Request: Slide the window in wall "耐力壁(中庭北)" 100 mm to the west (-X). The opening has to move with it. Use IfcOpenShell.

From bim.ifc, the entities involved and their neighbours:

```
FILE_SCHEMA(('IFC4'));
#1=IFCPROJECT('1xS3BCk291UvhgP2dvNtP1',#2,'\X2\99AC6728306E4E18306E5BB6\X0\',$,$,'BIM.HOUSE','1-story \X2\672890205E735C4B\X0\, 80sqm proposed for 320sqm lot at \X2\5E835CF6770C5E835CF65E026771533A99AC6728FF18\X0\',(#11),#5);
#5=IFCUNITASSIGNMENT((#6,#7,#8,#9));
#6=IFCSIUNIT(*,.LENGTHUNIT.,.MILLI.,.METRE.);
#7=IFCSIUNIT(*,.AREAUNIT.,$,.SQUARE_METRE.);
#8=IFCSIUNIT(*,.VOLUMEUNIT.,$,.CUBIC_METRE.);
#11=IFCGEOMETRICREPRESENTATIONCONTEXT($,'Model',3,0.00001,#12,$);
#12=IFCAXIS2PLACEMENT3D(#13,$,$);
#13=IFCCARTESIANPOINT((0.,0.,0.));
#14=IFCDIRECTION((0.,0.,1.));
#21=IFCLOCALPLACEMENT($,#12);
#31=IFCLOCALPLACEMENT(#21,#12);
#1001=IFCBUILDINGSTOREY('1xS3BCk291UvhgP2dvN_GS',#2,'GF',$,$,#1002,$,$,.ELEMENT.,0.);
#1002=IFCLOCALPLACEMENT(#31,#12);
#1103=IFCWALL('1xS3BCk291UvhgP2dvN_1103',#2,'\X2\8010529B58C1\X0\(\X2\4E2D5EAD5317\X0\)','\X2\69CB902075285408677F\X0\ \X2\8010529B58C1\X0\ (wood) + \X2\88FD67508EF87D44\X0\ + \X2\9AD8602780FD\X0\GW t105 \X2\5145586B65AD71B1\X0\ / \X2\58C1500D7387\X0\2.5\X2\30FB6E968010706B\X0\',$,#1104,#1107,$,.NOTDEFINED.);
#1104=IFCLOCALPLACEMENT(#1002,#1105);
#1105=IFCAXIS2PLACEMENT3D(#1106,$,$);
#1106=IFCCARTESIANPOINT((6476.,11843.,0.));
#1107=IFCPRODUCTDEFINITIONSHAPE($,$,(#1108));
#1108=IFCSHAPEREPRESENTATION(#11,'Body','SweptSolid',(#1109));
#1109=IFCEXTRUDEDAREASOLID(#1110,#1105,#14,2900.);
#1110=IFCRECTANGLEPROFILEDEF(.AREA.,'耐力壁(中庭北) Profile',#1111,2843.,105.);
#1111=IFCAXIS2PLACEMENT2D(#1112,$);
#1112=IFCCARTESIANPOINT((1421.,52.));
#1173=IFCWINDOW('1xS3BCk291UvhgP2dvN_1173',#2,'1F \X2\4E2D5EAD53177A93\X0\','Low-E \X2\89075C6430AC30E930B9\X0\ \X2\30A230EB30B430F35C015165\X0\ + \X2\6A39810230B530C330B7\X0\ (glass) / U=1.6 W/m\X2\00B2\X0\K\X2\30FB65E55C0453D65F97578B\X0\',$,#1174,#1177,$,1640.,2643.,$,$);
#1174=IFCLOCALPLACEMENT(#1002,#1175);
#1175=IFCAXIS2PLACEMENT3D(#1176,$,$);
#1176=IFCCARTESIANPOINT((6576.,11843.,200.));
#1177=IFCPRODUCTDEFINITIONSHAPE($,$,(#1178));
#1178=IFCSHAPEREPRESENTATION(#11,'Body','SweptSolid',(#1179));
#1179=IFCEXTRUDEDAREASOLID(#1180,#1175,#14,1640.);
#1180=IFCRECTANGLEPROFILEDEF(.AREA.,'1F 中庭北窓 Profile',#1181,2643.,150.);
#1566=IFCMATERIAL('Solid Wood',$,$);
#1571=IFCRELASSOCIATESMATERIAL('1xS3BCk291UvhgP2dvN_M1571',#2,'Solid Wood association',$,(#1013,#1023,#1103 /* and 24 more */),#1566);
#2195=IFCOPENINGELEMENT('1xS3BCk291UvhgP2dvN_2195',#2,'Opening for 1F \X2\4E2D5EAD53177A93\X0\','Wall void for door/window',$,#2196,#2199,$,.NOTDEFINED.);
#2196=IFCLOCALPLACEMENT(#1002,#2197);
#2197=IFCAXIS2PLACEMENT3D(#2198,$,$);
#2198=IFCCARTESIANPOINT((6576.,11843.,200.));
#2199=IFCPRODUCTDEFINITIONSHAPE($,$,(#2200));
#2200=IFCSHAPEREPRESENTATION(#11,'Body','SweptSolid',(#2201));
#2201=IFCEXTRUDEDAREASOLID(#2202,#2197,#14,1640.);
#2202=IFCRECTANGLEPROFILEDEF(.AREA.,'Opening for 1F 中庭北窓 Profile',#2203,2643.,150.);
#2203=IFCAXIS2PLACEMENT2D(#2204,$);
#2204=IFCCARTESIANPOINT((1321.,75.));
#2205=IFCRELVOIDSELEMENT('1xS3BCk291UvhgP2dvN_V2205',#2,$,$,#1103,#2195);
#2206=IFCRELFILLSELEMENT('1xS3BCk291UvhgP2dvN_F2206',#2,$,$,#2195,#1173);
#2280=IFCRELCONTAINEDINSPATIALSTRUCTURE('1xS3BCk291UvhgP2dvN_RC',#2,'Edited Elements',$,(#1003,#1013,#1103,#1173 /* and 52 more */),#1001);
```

```python
import ifcopenshell
import ifcopenshell.api.geometry
import ifcopenshell.util.placement
import ifcopenshell.util.unit

model = ifcopenshell.open("bim.ifc")
unit_scale = ifcopenshell.util.unit.calculate_unit_scale(model)

window = model.by_guid("1xS3BCk291UvhgP2dvN_1173")
opening = window.FillsVoids[0].RelatingOpeningElement
wall = opening.VoidsElements[0].RelatingBuildingElement

wall_matrix = ifcopenshell.util.placement.get_local_placement(wall.ObjectPlacement)
shift = wall_matrix[:3, 0] * -0.1 / unit_scale
before = ifcopenshell.util.placement.get_local_placement(window.ObjectPlacement)[:3, 3].copy()

# The window is not placed relative to its opening, so move both.
for product in (opening, window):
    matrix = ifcopenshell.util.placement.get_local_placement(product.ObjectPlacement)
    matrix[:3, 3] += shift
    ifcopenshell.api.geometry.edit_object_placement(model, product=product, matrix=matrix, is_si=False)

after = ifcopenshell.util.placement.get_local_placement(window.ObjectPlacement)[:3, 3]
print("window moved by", (after - before).round(3) + 0.0)

model.write("bim_updated.ifc")
```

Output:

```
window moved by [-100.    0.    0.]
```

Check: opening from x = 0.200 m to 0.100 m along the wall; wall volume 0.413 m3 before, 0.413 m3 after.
